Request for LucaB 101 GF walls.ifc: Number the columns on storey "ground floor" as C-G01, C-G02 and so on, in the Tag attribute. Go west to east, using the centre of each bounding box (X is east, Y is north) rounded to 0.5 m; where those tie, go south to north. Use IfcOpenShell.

First a look at what the model holds.

```python
import ifcopenshell
import ifcopenshell.util.element
import ifcopenshell.util.placement

model = ifcopenshell.open("LucaB 101 GF walls.ifc")
print(model.schema)
storey = next(s for s in model.by_type("IfcBuildingStorey") if s.Name == "ground floor")
columns = [e for e in ifcopenshell.util.element.get_decomposition(storey) if e.is_a("IfcColumn")]
for e in sorted(columns, key=lambda e: e.id()):
    origin = ifcopenshell.util.placement.get_local_placement(e.ObjectPlacement)[:3, 3]
    print(e.id(), e.Tag, e.Name, origin.round(2) + 0.0, sep=" | ")
```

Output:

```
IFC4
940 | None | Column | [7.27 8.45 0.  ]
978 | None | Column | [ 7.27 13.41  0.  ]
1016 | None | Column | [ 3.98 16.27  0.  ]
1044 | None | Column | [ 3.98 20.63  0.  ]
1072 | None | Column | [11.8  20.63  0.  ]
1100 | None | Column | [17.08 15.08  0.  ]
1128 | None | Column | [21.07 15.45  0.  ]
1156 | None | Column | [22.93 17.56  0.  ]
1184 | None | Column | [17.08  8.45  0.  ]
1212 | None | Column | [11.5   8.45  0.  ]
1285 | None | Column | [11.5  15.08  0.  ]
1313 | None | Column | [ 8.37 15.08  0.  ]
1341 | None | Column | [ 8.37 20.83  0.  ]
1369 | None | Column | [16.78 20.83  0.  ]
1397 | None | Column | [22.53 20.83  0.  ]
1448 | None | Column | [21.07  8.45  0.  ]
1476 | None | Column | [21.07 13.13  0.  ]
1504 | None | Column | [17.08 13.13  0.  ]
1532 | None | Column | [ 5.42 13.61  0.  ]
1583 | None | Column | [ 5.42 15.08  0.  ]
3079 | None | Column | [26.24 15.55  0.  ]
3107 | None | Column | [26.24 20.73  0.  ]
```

```python
import ifcopenshell
import ifcopenshell.geom
import ifcopenshell.util.element
import ifcopenshell.util.shape

model = ifcopenshell.open("LucaB 101 GF walls.ifc")
settings = ifcopenshell.geom.settings()
settings.set("use-world-coords", True)


def centre(element):
    shape = ifcopenshell.geom.create_shape(settings, element)
    return ifcopenshell.util.shape.get_bbox_centroid(shape.geometry)


storey = next(s for s in model.by_type("IfcBuildingStorey") if s.Name == "ground floor")
columns = [e for e in ifcopenshell.util.element.get_decomposition(storey) if e.is_a("IfcColumn")]

# Insertion points can sit at a corner or the storey origin, so sort by the geometry (in metres).
centres = {e: centre(e) for e in columns}
columns.sort(key=lambda e: (round(centres[e][0] / 0.5), centres[e][1]))

for i, e in enumerate(columns, start=1):
    number = f"C-G{i:02d}"
    e.Tag = number
    print(e.id(), number)

model.write("LucaB 101 GF walls_updated.ifc")
```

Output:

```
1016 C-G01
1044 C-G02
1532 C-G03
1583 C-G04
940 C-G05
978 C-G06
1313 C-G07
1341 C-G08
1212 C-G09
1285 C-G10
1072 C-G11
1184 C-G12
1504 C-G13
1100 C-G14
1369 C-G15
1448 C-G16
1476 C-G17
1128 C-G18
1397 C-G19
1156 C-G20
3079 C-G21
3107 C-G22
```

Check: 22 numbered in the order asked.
